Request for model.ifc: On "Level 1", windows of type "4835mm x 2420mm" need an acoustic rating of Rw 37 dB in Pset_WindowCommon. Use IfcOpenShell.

First a look at what the model holds.

```python
import ifcopenshell
import ifcopenshell.util.element

model = ifcopenshell.open("model.ifc")
print(model.schema)
storey = next(s for s in model.by_type("IfcBuildingStorey") if s.Name == "Level 1")
windows = [e for e in ifcopenshell.util.element.get_decomposition(storey) if e.is_a("IfcWindow")]
seen = {}
for e in windows:
    element_type = ifcopenshell.util.element.get_type(e)
    key = (element_type.Name if element_type != e and element_type else None, ifcopenshell.util.element.get_pset(e, "Pset_WindowCommon", "AcousticRating"))
    seen[key] = seen.get(key, 0) + 1
for (name, value), count in sorted(seen.items(), key=str):
    print(count, "x", name, "|", value)
```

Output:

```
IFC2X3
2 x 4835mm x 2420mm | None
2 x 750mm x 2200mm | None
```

```python
import ifcopenshell
import ifcopenshell.api.pset
import ifcopenshell.util.element

model = ifcopenshell.open("model.ifc")

storey = next(s for s in model.by_type("IfcBuildingStorey") if s.Name == "Level 1")
windows = [e for e in ifcopenshell.util.element.get_decomposition(storey) if e.is_a("IfcWindow")]

count = 0
for e in windows:
    element_type = ifcopenshell.util.element.get_type(e)
    if element_type in (None, e) or element_type.Name != "4835mm x 2420mm":
        continue
    # add_pset returns the element's existing set when there is one.
    pset = ifcopenshell.api.pset.add_pset(model, product=e, name="Pset_WindowCommon")
    ifcopenshell.api.pset.edit_pset(model, pset=pset, properties={"AcousticRating": "Rw 37 dB"})
    count += 1

print(count, "windows updated")

model.write("model_updated.ifc")
```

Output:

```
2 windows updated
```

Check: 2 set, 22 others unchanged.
